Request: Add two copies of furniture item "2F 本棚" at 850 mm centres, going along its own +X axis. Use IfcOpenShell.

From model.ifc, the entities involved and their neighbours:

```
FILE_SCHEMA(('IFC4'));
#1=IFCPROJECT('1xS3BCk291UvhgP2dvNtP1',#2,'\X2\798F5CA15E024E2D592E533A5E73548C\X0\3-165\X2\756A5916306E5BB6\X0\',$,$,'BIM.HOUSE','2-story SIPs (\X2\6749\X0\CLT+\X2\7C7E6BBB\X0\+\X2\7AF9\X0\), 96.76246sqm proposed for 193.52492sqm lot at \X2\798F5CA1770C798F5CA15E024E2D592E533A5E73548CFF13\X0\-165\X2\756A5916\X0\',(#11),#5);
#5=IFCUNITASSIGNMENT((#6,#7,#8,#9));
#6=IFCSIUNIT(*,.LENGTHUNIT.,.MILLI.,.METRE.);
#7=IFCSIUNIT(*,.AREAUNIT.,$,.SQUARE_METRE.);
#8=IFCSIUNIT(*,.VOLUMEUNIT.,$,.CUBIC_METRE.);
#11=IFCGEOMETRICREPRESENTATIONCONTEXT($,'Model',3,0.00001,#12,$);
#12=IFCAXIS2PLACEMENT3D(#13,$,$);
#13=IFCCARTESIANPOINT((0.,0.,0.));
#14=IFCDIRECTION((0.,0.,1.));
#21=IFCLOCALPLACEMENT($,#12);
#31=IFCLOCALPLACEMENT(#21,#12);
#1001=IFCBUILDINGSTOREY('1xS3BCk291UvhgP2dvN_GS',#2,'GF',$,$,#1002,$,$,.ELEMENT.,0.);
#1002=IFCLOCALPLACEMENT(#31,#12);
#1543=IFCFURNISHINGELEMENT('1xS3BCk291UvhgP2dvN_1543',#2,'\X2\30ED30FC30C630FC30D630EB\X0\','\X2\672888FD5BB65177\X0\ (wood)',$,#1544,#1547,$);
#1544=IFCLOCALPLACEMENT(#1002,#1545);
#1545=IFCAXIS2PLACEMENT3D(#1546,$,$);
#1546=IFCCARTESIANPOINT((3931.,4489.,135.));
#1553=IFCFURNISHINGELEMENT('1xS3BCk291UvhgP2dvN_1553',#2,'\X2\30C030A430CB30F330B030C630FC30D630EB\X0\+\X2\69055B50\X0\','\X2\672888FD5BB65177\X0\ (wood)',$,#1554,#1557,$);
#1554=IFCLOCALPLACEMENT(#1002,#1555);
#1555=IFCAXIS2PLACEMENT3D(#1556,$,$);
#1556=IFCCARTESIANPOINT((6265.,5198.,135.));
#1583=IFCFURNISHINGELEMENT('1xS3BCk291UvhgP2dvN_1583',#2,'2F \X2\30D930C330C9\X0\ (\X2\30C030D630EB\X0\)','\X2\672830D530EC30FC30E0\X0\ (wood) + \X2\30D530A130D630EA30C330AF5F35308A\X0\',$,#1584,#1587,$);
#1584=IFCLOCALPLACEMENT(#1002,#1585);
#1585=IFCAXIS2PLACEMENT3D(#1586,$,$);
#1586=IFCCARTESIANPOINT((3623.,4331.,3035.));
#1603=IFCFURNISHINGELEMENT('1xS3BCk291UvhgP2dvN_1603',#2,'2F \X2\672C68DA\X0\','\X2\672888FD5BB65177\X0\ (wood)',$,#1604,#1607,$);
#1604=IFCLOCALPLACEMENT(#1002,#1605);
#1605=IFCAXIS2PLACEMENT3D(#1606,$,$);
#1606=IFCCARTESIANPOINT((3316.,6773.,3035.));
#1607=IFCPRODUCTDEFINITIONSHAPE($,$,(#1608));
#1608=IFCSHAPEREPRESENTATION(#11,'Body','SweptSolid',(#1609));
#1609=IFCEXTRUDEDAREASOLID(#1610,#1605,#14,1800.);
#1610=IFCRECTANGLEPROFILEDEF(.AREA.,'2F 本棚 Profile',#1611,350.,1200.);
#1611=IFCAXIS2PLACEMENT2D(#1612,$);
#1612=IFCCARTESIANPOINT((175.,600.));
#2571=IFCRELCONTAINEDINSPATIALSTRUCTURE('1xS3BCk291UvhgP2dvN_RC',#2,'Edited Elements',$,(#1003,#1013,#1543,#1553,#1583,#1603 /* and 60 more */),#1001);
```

```python
import ifcopenshell
import ifcopenshell.api.geometry
import ifcopenshell.api.root
import ifcopenshell.util.element
import ifcopenshell.util.placement
import ifcopenshell.util.unit

model = ifcopenshell.open("model.ifc")
unit_scale = ifcopenshell.util.unit.calculate_unit_scale(model)


def reuse_history(source, copy):
    """copy_class also copies each property set's owner history, people and application; keep the originals."""
    for rel in copy.IsDefinedBy:
        if rel.is_a("IfcRelDefinesByProperties") and (history := rel.RelatingPropertyDefinition.OwnerHistory):
            rel.RelatingPropertyDefinition.OwnerHistory = source.OwnerHistory
            ifcopenshell.util.element.remove_deep2(model, history)


source = model.by_guid("1xS3BCk291UvhgP2dvN_1603")
base = ifcopenshell.util.placement.get_local_placement(source.ObjectPlacement)
step = base[:3, 0] * 0.85 / unit_scale

for i in range(1, 3):
    copy = ifcopenshell.api.root.copy_class(model, product=source)
    copy.Representation = ifcopenshell.util.element.copy_deep(
        model, source.Representation, exclude=["IfcGeometricRepresentationContext", "IfcRepresentationMap"]
    )
    reuse_history(source, copy)
    matrix = base.copy()
    matrix[:3, 3] += i * step
    print("added at", matrix[:3, 3].round(3) + 0.0)
    ifcopenshell.api.geometry.edit_object_placement(model, product=copy, matrix=matrix, is_si=False)

model.write("model_edited.ifc")
```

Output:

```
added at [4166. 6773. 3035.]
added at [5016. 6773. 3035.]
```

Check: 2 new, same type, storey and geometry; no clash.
